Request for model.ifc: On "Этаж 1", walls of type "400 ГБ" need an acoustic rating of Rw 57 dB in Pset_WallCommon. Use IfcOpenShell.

First a look at what the model holds.

```python
import ifcopenshell
import ifcopenshell.util.element

model = ifcopenshell.open("model.ifc")
print(model.schema)
storey = next(s for s in model.by_type("IfcBuildingStorey") if s.Name == "Этаж 1")
walls = [e for e in ifcopenshell.util.element.get_decomposition(storey) if e.is_a("IfcWall")]
seen = {}
for e in walls:
    element_type = ifcopenshell.util.element.get_type(e)
    key = (element_type.Name if element_type != e and element_type else None, ifcopenshell.util.element.get_pset(e, "Pset_WallCommon", "AcousticRating"))
    seen[key] = seen.get(key, 0) + 1
for (name, value), count in sorted(seen.items(), key=str):
    print(count, "x", name, "|", value)
```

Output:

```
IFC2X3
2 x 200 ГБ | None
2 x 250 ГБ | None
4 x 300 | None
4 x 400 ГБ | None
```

```python
import ifcopenshell
import ifcopenshell.api.pset
import ifcopenshell.util.element

model = ifcopenshell.open("model.ifc")

storey = next(s for s in model.by_type("IfcBuildingStorey") if s.Name == "Этаж 1")
walls = [e for e in ifcopenshell.util.element.get_decomposition(storey) if e.is_a("IfcWall")]

count = 0
for e in walls:
    element_type = ifcopenshell.util.element.get_type(e)
    if element_type in (None, e) or element_type.Name != "400 ГБ":
        continue
    # add_pset returns the element's existing set when there is one.
    pset = ifcopenshell.api.pset.add_pset(model, product=e, name="Pset_WallCommon")
    ifcopenshell.api.pset.edit_pset(model, pset=pset, properties={"AcousticRating": "Rw 57 dB"})
    count += 1

print(count, "walls updated")

model.write("model_v2.ifc")
```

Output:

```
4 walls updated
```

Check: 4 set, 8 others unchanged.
